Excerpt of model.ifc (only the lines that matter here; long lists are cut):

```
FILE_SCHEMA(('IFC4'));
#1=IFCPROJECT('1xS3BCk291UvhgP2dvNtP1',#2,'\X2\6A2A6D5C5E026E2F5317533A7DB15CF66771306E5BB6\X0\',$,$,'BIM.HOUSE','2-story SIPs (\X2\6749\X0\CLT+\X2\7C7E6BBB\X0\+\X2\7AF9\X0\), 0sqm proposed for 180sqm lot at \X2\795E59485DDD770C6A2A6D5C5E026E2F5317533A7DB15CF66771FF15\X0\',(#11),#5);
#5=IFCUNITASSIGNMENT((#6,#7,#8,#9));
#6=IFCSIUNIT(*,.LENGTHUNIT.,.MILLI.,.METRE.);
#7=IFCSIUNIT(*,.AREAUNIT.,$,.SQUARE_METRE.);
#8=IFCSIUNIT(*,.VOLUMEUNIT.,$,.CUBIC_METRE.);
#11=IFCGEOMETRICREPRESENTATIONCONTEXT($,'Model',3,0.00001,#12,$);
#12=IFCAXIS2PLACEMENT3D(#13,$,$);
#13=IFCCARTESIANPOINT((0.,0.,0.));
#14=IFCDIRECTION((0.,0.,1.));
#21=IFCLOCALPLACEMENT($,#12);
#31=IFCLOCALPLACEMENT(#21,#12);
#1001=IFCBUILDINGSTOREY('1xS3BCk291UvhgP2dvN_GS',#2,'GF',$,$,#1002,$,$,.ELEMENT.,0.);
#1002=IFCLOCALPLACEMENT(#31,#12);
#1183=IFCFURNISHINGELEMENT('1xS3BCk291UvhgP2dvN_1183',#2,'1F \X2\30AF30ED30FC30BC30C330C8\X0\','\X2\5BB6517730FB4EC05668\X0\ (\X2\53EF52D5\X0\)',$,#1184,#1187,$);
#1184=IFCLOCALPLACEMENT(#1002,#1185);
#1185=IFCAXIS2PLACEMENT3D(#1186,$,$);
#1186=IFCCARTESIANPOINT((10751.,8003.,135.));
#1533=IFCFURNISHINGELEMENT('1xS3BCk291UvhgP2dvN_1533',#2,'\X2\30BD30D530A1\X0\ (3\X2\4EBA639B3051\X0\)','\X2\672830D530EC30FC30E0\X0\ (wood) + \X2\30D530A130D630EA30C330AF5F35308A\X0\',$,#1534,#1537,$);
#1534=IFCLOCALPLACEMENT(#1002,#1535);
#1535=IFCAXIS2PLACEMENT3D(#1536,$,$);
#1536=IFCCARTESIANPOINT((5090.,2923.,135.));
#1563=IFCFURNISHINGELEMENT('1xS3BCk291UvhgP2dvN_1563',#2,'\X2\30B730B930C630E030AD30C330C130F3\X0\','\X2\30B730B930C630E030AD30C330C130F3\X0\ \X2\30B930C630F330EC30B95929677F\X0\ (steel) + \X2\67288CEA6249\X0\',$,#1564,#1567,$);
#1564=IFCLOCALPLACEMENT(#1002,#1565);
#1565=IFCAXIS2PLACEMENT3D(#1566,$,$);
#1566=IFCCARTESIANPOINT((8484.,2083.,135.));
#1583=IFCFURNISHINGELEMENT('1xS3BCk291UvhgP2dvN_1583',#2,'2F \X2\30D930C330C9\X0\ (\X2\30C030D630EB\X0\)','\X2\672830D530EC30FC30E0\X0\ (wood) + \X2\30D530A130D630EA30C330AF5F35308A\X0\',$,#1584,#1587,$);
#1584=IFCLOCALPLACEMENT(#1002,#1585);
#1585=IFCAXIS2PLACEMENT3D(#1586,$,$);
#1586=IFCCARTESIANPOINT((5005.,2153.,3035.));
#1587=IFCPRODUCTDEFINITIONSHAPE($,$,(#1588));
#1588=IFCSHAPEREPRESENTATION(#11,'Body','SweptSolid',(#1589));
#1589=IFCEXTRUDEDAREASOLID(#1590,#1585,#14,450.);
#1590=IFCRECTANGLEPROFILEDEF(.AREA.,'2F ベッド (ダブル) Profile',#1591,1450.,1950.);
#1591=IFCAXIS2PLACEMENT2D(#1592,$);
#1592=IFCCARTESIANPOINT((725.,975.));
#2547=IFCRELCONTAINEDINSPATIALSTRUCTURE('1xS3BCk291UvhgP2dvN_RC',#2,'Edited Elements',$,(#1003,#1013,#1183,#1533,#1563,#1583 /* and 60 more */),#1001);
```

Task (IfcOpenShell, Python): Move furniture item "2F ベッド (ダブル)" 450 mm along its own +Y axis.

```python
import ifcopenshell
import ifcopenshell.api.geometry
import ifcopenshell.util.placement

model = ifcopenshell.open("model.ifc")

item = model.by_guid("1xS3BCk291UvhgP2dvN_1583")
matrix = ifcopenshell.util.placement.get_local_placement(item.ObjectPlacement)
matrix[:3, 3] += matrix[:3, 1] * 450.0
ifcopenshell.api.geometry.edit_object_placement(model, product=item, matrix=matrix, is_si=False)

print(ifcopenshell.util.placement.get_local_placement(item.ObjectPlacement).round(3) + 0.0)

model.write("model_rev.ifc")
```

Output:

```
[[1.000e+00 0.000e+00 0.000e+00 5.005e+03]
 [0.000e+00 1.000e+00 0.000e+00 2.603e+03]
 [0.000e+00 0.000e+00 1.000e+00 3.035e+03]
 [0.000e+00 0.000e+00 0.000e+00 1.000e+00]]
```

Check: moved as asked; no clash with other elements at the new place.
